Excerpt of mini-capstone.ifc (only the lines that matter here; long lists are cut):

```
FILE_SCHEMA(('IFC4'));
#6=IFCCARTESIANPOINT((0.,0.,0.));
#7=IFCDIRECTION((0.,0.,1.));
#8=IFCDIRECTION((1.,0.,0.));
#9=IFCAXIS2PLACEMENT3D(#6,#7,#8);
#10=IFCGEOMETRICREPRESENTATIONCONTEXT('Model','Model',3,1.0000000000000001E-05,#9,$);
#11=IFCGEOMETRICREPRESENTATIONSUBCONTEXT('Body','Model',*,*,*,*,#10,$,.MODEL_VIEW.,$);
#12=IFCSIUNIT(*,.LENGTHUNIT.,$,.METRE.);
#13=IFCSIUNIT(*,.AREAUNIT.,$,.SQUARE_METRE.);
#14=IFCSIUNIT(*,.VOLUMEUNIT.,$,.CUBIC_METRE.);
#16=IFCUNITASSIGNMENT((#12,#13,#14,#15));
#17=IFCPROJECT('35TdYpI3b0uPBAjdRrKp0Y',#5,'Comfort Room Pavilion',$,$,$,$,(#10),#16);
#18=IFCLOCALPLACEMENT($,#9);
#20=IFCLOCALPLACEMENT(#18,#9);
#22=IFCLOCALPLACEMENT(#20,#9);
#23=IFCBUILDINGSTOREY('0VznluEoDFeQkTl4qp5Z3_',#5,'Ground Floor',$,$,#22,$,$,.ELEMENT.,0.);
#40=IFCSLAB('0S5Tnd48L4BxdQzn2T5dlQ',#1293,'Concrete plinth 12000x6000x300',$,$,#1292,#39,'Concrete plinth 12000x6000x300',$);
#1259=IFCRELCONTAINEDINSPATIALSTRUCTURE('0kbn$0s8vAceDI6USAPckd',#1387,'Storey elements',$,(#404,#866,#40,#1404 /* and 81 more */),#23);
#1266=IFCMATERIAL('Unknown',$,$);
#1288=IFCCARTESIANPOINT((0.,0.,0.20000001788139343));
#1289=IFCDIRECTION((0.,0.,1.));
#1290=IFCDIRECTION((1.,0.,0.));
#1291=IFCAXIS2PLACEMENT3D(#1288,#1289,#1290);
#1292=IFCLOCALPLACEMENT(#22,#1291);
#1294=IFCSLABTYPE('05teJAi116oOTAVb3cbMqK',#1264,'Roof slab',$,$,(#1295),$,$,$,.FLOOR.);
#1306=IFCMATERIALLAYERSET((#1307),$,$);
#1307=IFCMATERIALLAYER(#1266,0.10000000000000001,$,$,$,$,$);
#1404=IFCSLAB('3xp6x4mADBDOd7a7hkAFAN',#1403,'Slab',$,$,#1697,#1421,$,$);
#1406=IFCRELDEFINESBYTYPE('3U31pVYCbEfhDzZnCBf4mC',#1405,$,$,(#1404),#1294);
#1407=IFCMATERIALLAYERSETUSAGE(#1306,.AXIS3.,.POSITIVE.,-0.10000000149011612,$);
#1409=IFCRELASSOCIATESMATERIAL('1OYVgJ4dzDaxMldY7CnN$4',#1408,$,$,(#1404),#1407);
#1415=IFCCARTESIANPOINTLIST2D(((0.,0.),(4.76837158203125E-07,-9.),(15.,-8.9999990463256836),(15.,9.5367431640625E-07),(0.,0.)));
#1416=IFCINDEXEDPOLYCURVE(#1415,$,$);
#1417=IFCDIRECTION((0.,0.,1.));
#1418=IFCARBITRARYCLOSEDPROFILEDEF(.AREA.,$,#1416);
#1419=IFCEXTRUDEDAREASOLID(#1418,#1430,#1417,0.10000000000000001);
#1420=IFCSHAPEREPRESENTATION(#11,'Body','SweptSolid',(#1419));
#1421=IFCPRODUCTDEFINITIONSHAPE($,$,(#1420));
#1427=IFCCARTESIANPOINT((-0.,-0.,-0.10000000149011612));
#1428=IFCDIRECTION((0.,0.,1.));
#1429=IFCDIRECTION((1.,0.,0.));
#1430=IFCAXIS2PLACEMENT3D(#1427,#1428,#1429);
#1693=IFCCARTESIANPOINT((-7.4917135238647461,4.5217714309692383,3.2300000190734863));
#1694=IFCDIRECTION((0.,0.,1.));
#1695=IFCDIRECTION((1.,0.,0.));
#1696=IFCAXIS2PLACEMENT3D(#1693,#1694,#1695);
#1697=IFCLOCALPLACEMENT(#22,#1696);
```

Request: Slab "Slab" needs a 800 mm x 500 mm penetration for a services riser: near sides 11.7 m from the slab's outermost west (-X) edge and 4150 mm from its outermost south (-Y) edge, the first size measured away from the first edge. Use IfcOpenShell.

```python
import numpy as np
import ifcopenshell
import ifcopenshell.api.feature
import ifcopenshell.api.geometry
import ifcopenshell.api.root
import ifcopenshell.geom
import ifcopenshell.util.placement
import ifcopenshell.util.representation
import ifcopenshell.util.shape
import ifcopenshell.util.unit

model = ifcopenshell.open("mini-capstone.ifc")
unit_scale = ifcopenshell.util.unit.calculate_unit_scale(model)
settings = ifcopenshell.geom.settings()


def volume(element):
    """Net volume in cubic metres, openings subtracted."""
    shape = ifcopenshell.geom.create_shape(settings, element)
    return ifcopenshell.util.shape.get_volume(shape.geometry)


slab = model.by_id(1404)
before = volume(slab)

# Extent in the slab's own axes, in metres. The edges named are its -X and -Y sides.
slab_shape = ifcopenshell.geom.create_shape(settings, slab)
vertices = ifcopenshell.util.shape.get_vertices(slab_shape.geometry)
x_min, y_min, bottom = vertices.min(axis=0)
top = vertices[:, 2].max()

opening = ifcopenshell.api.root.create_entity(model, ifc_class="IfcOpeningElement", name="Services riser opening", predefined_type="OPENING")
context = ifcopenshell.util.representation.get_context(model, "Model", "Body", "MODEL_VIEW")
width, depth = 0.8, 0.5
outline = [(0.0, 0.0), (width, 0.0), (width, depth), (0.0, depth), (0.0, 0.0)]
# Overshoot both faces by 50 mm so the cut is clean.
shape = ifcopenshell.api.geometry.add_slab_representation(
    model, context=context, depth=top - bottom + 0.1, polyline=outline
)
ifcopenshell.api.geometry.assign_representation(model, product=opening, representation=shape)

matrix = ifcopenshell.util.placement.get_local_placement(slab.ObjectPlacement)
matrix[:, 3] = matrix @ np.append(np.array([x_min + 11.7, y_min + 4.15, bottom - 0.05]) / unit_scale, 1.0)
ifcopenshell.api.geometry.edit_object_placement(model, product=opening, matrix=matrix, is_si=False)
ifcopenshell.api.feature.add_feature(model, feature=opening, element=slab)

after = volume(slab)

print(f"slab volume {before:.3f} -> {after:.3f} m3")

model.write("mini-capstone-out.ifc")
```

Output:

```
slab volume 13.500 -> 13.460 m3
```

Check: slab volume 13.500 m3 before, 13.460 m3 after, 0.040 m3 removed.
